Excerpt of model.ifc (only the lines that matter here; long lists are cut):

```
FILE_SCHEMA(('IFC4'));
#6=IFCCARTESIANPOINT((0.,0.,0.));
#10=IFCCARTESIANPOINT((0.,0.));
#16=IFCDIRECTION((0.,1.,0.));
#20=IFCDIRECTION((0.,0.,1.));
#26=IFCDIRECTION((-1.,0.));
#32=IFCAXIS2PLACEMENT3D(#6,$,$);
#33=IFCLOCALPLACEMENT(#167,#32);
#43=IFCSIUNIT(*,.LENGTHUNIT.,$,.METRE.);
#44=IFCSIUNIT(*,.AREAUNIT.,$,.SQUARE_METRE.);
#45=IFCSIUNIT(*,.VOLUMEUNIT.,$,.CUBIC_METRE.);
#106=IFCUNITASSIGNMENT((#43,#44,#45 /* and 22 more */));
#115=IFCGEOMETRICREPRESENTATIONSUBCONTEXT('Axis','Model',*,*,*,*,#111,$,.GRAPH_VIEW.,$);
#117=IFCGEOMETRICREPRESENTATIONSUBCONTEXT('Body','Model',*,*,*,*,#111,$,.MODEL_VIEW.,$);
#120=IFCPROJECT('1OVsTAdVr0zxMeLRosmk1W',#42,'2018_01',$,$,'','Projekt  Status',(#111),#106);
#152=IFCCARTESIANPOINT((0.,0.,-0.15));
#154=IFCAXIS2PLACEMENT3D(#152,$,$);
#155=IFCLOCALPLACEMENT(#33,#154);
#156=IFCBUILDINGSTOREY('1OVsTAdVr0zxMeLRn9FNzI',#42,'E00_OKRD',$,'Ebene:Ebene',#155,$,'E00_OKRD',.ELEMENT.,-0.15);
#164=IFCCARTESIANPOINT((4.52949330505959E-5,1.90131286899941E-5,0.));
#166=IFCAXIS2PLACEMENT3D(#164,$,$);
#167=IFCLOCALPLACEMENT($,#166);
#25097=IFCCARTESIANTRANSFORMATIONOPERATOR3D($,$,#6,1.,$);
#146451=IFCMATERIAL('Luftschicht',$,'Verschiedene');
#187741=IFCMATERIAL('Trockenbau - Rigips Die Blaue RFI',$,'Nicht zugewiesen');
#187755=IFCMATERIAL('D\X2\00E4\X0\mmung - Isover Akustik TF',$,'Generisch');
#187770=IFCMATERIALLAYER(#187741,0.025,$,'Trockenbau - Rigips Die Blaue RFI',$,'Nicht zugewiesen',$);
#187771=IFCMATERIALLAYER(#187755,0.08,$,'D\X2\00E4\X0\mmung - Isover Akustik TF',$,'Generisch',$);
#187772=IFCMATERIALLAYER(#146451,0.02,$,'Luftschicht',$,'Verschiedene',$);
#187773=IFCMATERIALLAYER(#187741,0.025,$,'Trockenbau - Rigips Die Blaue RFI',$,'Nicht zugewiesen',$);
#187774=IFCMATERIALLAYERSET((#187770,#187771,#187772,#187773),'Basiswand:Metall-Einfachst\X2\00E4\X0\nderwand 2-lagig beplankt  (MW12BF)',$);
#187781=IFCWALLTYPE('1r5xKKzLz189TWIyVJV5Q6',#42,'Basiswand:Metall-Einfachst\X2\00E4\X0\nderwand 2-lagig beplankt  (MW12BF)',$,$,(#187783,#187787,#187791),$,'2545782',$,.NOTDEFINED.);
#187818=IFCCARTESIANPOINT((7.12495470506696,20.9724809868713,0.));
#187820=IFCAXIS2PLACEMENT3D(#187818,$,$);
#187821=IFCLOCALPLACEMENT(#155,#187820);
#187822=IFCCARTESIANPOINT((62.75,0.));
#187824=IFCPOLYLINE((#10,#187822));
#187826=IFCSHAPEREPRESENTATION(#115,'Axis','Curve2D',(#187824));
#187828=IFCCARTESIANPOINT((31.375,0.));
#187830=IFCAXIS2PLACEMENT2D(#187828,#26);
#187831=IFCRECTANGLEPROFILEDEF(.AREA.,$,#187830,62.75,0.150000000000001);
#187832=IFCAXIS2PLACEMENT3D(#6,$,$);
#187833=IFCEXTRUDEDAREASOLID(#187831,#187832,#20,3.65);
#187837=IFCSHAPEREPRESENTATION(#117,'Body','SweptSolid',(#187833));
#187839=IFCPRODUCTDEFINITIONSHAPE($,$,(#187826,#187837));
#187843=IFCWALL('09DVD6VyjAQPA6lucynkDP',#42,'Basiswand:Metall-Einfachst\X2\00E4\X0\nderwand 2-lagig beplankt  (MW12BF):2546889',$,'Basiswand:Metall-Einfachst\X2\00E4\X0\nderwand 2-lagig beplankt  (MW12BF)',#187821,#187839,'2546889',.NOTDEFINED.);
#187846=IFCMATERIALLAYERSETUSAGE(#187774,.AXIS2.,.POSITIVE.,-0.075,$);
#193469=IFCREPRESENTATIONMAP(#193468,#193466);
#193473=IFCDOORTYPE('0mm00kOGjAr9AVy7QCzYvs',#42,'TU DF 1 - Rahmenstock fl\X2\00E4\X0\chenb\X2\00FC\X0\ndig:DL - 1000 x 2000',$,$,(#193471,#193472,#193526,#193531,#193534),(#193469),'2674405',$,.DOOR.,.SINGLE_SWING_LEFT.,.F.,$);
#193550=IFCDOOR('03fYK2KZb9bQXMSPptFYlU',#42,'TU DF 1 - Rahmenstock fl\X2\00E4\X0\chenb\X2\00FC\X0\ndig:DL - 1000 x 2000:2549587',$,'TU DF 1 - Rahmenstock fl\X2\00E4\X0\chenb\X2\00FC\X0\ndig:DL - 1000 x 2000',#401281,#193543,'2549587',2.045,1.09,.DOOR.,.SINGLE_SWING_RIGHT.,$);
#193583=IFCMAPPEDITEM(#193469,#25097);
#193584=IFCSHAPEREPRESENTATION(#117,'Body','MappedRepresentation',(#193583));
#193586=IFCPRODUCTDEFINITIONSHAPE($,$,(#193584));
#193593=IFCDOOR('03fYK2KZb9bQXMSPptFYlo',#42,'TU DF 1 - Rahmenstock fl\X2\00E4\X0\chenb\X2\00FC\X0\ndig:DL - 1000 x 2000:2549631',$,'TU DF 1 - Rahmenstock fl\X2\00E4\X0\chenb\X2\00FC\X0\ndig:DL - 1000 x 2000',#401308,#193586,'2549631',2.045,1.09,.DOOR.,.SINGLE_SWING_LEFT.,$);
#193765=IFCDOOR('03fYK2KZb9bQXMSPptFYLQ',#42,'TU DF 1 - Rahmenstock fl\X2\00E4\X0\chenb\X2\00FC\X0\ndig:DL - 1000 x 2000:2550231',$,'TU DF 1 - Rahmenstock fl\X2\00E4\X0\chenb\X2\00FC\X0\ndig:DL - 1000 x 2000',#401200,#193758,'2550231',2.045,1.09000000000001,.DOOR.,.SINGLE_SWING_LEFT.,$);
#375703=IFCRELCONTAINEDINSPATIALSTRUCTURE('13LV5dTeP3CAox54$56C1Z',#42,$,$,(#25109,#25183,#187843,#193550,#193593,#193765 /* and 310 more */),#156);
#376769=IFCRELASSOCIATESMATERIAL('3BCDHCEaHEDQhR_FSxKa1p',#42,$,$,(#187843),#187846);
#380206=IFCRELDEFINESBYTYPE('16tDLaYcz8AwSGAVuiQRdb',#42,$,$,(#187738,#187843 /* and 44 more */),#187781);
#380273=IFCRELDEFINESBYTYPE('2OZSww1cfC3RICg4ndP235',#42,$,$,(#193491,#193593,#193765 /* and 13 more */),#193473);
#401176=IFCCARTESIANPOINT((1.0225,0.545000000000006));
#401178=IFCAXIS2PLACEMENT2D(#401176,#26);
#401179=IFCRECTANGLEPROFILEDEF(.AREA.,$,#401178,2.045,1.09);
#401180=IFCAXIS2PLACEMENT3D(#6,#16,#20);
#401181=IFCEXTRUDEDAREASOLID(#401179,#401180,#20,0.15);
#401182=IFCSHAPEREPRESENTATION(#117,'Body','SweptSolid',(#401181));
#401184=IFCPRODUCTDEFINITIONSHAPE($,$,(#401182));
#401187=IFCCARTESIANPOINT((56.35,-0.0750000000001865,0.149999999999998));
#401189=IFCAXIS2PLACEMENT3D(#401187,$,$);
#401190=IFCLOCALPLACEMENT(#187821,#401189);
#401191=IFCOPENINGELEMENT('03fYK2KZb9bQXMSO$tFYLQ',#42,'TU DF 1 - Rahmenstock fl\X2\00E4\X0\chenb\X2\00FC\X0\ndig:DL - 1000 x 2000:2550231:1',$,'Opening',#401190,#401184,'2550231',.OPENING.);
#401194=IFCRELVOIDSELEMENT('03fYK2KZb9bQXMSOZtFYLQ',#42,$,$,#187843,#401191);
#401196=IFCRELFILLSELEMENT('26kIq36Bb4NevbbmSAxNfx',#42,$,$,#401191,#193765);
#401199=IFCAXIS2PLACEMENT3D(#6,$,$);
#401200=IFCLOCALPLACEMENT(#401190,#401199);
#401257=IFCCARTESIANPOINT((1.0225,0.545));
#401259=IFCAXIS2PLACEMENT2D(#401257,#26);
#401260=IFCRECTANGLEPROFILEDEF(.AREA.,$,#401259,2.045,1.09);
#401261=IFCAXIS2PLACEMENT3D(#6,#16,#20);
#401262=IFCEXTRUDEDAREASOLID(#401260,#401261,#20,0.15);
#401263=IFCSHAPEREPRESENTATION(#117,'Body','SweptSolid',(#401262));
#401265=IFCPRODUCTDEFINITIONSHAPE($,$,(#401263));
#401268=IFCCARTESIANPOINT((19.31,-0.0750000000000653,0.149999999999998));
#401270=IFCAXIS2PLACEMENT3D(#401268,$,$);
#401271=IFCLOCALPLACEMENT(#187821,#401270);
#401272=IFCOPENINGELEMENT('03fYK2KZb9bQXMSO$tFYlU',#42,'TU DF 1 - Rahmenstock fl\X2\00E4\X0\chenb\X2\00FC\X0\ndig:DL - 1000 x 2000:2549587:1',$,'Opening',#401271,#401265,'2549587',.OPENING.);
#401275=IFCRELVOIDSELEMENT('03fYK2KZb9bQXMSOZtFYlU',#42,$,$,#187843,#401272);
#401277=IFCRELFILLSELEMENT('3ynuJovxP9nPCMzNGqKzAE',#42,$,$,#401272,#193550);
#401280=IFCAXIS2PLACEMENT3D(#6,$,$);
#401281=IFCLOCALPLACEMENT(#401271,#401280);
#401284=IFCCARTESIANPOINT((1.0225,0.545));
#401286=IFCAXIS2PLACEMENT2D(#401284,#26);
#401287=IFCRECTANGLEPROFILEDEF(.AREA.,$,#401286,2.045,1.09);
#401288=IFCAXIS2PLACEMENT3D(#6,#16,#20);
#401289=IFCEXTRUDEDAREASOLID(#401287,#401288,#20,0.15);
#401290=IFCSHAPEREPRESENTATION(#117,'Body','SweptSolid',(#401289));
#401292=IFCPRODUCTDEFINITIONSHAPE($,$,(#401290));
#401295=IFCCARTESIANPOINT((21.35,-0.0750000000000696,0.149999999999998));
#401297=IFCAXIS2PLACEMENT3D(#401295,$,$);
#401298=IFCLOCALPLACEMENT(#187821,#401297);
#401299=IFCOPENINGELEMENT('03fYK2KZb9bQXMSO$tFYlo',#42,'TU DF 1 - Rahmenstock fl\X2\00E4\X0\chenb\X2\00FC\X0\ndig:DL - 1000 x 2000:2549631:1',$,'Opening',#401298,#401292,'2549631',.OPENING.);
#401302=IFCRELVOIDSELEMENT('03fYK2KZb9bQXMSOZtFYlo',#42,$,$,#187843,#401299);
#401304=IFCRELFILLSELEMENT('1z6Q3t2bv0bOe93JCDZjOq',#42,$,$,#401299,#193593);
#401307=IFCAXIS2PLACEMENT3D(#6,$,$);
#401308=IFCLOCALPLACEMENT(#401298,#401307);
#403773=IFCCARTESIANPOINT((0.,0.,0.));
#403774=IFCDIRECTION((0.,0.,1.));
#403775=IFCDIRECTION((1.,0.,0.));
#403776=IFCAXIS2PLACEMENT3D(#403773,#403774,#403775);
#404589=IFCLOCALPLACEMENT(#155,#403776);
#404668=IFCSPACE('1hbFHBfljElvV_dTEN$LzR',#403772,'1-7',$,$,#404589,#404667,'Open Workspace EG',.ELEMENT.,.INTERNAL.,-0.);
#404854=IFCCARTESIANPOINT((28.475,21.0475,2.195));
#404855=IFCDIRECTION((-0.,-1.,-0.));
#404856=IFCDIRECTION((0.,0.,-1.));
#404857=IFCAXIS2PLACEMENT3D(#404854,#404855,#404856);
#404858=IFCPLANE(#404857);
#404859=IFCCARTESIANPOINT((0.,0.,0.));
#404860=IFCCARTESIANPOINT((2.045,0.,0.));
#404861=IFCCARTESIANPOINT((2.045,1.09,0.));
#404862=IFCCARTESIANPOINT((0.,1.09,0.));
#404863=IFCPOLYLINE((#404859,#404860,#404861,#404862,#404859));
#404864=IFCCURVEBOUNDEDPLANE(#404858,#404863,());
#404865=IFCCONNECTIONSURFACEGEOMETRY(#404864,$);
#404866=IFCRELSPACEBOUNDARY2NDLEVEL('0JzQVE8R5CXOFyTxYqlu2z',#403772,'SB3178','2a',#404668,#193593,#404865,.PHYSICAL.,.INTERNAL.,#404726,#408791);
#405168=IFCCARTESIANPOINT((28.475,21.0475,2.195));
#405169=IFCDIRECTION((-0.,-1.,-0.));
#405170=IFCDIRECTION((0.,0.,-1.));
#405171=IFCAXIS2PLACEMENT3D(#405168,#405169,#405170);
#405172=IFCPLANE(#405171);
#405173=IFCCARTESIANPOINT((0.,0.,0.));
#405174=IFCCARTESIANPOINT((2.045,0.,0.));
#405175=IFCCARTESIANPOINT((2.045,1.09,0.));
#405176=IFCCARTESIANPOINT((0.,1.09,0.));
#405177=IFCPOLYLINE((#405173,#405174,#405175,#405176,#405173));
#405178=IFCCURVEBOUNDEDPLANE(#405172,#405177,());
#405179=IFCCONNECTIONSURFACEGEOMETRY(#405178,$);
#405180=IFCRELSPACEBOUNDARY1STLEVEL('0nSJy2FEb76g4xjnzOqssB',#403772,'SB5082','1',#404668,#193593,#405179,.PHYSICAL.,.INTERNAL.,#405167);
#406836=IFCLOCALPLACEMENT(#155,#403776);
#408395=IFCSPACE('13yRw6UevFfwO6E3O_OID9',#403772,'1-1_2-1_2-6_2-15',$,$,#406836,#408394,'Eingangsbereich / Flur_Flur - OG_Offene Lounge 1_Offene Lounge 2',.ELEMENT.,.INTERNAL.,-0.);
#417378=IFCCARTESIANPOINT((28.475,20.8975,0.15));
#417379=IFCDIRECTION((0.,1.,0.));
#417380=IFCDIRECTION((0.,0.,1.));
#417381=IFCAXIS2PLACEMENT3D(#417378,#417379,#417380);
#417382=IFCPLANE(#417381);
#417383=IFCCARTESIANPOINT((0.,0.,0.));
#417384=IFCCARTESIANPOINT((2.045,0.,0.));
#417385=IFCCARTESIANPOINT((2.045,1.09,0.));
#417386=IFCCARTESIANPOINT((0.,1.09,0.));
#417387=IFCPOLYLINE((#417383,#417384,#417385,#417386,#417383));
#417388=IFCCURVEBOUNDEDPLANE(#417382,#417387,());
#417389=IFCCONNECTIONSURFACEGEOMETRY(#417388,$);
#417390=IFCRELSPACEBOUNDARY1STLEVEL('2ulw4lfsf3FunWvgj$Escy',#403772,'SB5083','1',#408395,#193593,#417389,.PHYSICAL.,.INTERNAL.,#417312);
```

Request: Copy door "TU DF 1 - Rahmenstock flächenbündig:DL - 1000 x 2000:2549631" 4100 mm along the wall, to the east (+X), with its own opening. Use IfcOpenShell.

```python
import numpy as np
import ifcopenshell
import ifcopenshell.api.feature
import ifcopenshell.api.geometry
import ifcopenshell.api.root
import ifcopenshell.geom
import ifcopenshell.util.element
import ifcopenshell.util.placement
import ifcopenshell.util.shape

model = ifcopenshell.open("model.ifc")
settings = ifcopenshell.geom.settings()


def volume(element):
    """Net volume in cubic metres, openings subtracted."""
    shape = ifcopenshell.geom.create_shape(settings, element)
    return ifcopenshell.util.shape.get_volume(shape.geometry)


def reuse_history(source, copy):
    """copy_class also copies each property set's owner history, people and application; keep the originals."""
    for rel in copy.IsDefinedBy:
        if rel.is_a("IfcRelDefinesByProperties") and (history := rel.RelatingPropertyDefinition.OwnerHistory):
            rel.RelatingPropertyDefinition.OwnerHistory = source.OwnerHistory
            ifcopenshell.util.element.remove_deep2(model, history)


door = model.by_guid("03fYK2KZb9bQXMSPptFYlo")
opening = door.FillsVoids[0].RelatingOpeningElement
wall = opening.VoidsElements[0].RelatingBuildingElement
before = volume(wall)
shift = ifcopenshell.util.placement.get_local_placement(wall.ObjectPlacement)[:3, 0] * 4.1

# copy_class copies the void relationship, type, container and properties, but no geometry.
new_opening = ifcopenshell.api.root.copy_class(model, product=opening)
new_opening.Representation = ifcopenshell.util.element.copy_deep(
    model, opening.Representation, exclude=["IfcGeometricRepresentationContext", "IfcRepresentationMap"]
)
new_opening.Name = "TU DF 1 - Rahmenstock flächenbündig:DL - 1000 x 2000"
new_opening.Tag = None
new_door = ifcopenshell.api.root.copy_class(model, product=door)
new_door.Representation = ifcopenshell.util.element.copy_deep(
    model, door.Representation, exclude=["IfcGeometricRepresentationContext", "IfcRepresentationMap"]
)
new_door.Name = "TU DF 1 - Rahmenstock flächenbündig:DL - 1000 x 2000"
new_door.Tag = None
reuse_history(door, new_door)
ifcopenshell.api.feature.add_filling(model, opening=new_opening, element=new_door)

for old, new in ((opening, new_opening), (door, new_door)):
    matrix = ifcopenshell.util.placement.get_local_placement(old.ObjectPlacement)
    matrix[:3, 3] += shift
    ifcopenshell.api.geometry.edit_object_placement(model, product=new, matrix=matrix, is_si=False)

# The copied space boundaries still share their surfaces with the original.
for rel in new_door.ProvidesBoundaries:
    if rel.ConnectionGeometry:
        rel.ConnectionGeometry = ifcopenshell.util.element.copy_deep(model, rel.ConnectionGeometry)

# Space boundary surfaces are stored in each space's coordinates; move them too.
for rel in new_door.ProvidesBoundaries:
    if not rel.ConnectionGeometry:
        continue
    surface = rel.ConnectionGeometry.SurfaceOnRelatingElement.BasisSurface
    space_matrix = ifcopenshell.util.placement.get_local_placement(rel.RelatingSpace.ObjectPlacement)
    point = np.array(surface.Position.Location.Coordinates) + space_matrix[:3, :3].T @ shift
    surface.Position = model.createIfcAxis2Placement3D(
        model.createIfcCartesianPoint(point.tolist()), surface.Position.Axis, surface.Position.RefDirection
    )

after = volume(wall)

print(f"wall volume {before:.3f} -> {after:.3f} m3")

model.write("model_v2.ifc")
```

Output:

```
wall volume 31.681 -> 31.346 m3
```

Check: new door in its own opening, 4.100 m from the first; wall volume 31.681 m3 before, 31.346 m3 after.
